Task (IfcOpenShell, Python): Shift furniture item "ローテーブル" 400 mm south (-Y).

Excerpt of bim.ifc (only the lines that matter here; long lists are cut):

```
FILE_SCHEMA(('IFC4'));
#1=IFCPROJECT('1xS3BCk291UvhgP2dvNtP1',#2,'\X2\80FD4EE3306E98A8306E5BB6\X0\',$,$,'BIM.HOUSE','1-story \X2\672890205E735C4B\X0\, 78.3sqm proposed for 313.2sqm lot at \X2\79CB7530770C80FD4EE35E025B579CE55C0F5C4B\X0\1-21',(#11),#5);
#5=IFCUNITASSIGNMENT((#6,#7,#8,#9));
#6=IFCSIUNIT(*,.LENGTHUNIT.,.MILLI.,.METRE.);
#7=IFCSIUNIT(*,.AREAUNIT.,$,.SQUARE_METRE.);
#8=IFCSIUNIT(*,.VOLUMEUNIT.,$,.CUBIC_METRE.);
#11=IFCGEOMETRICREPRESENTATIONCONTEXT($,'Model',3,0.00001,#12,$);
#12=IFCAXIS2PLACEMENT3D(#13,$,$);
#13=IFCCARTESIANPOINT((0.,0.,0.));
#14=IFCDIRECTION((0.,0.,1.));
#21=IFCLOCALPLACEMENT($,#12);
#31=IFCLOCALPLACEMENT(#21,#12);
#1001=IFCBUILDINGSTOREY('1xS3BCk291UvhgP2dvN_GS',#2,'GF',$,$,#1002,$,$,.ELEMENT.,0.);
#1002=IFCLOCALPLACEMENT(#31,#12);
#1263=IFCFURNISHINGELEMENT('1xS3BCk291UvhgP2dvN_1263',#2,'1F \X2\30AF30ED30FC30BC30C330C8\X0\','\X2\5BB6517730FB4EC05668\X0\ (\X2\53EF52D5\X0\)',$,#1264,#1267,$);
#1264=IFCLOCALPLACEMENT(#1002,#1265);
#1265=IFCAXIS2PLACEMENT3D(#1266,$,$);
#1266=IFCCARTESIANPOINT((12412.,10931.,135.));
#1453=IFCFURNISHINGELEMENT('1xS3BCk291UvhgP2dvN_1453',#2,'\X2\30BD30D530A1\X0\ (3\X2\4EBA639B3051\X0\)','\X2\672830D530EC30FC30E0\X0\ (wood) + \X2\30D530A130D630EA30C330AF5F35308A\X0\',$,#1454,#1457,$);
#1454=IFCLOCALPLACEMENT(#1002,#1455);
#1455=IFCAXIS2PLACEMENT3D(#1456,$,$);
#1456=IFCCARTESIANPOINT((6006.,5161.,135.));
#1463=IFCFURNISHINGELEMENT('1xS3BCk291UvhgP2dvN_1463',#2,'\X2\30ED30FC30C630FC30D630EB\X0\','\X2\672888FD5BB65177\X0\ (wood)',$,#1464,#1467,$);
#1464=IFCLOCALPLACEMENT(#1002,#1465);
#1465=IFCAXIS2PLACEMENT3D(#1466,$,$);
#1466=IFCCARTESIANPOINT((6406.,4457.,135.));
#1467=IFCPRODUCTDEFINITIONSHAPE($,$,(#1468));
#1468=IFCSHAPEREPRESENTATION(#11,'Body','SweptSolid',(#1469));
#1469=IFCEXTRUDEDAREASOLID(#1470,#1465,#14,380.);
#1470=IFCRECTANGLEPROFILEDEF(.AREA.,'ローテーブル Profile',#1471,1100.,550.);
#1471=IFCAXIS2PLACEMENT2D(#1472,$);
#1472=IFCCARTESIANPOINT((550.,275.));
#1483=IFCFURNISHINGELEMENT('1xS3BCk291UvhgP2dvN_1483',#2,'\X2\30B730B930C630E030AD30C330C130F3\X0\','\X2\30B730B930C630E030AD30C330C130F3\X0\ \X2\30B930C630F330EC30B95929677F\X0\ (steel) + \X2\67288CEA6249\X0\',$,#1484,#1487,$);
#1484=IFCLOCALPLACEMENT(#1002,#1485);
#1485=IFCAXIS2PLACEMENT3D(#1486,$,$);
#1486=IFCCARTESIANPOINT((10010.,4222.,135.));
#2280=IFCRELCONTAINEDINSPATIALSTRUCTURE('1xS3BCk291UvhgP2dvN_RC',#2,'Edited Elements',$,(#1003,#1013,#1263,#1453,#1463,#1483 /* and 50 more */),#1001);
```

```python
import ifcopenshell
import ifcopenshell.api.geometry
import ifcopenshell.util.placement

model = ifcopenshell.open("bim.ifc")

item = model.by_id(1463)
matrix = ifcopenshell.util.placement.get_local_placement(item.ObjectPlacement)
matrix[1, 3] -= 400.0
ifcopenshell.api.geometry.edit_object_placement(model, product=item, matrix=matrix, is_si=False)

print(ifcopenshell.util.placement.get_local_placement(item.ObjectPlacement).round(3) + 0.0)

model.write("bim_v2.ifc")
```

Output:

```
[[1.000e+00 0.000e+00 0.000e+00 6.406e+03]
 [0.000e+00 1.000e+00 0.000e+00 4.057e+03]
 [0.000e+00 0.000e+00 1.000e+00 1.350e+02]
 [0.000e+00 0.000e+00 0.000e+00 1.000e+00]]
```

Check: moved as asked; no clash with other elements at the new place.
